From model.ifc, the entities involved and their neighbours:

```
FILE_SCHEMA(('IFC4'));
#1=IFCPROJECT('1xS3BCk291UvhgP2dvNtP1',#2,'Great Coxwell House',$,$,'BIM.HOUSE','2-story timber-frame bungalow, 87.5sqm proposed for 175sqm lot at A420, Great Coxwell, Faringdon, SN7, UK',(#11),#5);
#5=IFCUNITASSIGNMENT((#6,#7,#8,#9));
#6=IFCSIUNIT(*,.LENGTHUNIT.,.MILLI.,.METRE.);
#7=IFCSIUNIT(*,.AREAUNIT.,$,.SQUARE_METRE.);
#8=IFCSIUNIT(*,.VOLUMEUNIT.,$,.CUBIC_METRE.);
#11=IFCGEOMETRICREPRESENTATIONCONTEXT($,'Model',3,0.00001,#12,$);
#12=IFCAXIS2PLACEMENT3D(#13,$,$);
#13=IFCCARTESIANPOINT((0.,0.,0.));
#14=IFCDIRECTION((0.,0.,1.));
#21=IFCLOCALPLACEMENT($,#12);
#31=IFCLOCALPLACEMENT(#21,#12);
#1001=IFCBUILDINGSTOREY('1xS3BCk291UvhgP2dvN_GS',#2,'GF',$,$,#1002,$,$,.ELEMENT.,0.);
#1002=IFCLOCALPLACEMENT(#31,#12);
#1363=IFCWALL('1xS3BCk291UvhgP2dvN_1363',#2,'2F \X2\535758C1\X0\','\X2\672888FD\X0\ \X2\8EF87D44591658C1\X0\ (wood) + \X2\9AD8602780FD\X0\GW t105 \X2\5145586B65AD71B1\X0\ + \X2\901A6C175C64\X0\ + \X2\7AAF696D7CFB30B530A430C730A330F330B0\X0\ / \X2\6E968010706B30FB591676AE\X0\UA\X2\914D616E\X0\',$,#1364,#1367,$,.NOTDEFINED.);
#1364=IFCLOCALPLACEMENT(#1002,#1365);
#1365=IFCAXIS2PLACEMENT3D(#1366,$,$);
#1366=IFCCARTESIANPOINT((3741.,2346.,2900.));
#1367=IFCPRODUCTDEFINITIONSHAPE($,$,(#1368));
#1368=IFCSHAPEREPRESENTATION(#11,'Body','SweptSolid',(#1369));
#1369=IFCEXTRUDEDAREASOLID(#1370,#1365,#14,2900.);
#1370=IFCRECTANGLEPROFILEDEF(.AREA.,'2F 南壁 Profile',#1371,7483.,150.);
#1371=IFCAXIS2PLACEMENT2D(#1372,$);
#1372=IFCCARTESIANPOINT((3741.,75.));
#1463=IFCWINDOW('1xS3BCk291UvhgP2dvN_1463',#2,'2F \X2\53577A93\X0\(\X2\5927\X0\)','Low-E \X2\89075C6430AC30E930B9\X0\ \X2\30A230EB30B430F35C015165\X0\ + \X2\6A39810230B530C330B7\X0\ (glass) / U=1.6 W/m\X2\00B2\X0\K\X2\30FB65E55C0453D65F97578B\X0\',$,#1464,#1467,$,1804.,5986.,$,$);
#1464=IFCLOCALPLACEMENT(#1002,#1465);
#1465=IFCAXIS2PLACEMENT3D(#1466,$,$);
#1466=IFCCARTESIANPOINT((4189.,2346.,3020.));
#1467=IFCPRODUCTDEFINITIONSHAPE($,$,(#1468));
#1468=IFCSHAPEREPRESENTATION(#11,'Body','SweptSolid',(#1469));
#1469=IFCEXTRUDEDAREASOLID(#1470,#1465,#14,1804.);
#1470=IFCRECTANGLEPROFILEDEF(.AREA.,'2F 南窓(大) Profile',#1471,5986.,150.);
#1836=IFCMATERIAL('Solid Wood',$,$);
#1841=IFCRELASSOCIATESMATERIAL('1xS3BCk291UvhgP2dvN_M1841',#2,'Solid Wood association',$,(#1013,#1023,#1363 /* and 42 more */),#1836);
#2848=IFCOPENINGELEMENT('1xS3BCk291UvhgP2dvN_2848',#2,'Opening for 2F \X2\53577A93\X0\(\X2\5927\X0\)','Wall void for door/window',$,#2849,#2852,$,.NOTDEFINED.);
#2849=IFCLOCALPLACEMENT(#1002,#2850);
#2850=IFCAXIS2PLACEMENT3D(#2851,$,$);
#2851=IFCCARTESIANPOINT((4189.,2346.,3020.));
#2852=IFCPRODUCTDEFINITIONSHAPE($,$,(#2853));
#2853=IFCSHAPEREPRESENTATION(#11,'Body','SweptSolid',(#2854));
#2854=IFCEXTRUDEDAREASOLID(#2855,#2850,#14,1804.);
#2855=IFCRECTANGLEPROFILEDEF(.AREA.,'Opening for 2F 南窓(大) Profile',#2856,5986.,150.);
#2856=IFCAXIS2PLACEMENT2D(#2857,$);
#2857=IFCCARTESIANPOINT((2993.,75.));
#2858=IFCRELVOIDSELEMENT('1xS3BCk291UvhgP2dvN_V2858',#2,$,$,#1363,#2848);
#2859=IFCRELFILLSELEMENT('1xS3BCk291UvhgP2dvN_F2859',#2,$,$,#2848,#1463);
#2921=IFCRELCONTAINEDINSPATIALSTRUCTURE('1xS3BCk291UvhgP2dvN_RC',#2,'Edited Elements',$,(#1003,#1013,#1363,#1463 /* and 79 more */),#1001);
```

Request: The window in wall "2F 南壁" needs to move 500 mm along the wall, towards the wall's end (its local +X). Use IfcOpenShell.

```python
import ifcopenshell
import ifcopenshell.api.geometry
import ifcopenshell.util.placement
import ifcopenshell.util.unit

model = ifcopenshell.open("model.ifc")
unit_scale = ifcopenshell.util.unit.calculate_unit_scale(model)

window = model.by_guid("1xS3BCk291UvhgP2dvN_1463")
opening = window.FillsVoids[0].RelatingOpeningElement
wall = opening.VoidsElements[0].RelatingBuildingElement

wall_matrix = ifcopenshell.util.placement.get_local_placement(wall.ObjectPlacement)
shift = wall_matrix[:3, 0] * 0.5 / unit_scale
before = ifcopenshell.util.placement.get_local_placement(window.ObjectPlacement)[:3, 3].copy()

# The window is not placed relative to its opening, so move both.
for product in (opening, window):
    matrix = ifcopenshell.util.placement.get_local_placement(product.ObjectPlacement)
    matrix[:3, 3] += shift
    ifcopenshell.api.geometry.edit_object_placement(model, product=product, matrix=matrix, is_si=False)

after = ifcopenshell.util.placement.get_local_placement(window.ObjectPlacement)[:3, 3]
print("window moved by", (after - before).round(3) + 0.0)

model.write("model_edited.ifc")
```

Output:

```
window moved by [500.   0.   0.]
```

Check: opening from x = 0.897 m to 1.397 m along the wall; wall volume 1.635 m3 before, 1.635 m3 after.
